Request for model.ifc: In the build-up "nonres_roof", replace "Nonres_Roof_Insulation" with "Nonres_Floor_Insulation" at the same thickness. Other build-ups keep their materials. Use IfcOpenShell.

First a look at what the model holds.

```python
import ifcopenshell
import ifcopenshell.util.element

model = ifcopenshell.open("model.ifc")
print(model.schema)
for layer_set in model.by_type("IfcMaterialLayerSet"):
    if layer_set.LayerSetName == "nonres_roof":
        for layer in layer_set.MaterialLayers:
            print(layer.id(), layer.Material and layer.Material.Name, layer.LayerThickness, sep=" | ")
        print(len(ifcopenshell.util.element.get_elements_by_material(model, layer_set)), "elements and types use it")
print(sorted(m.Name for m in model.by_type("IfcMaterial") if m.Name)[:60])
```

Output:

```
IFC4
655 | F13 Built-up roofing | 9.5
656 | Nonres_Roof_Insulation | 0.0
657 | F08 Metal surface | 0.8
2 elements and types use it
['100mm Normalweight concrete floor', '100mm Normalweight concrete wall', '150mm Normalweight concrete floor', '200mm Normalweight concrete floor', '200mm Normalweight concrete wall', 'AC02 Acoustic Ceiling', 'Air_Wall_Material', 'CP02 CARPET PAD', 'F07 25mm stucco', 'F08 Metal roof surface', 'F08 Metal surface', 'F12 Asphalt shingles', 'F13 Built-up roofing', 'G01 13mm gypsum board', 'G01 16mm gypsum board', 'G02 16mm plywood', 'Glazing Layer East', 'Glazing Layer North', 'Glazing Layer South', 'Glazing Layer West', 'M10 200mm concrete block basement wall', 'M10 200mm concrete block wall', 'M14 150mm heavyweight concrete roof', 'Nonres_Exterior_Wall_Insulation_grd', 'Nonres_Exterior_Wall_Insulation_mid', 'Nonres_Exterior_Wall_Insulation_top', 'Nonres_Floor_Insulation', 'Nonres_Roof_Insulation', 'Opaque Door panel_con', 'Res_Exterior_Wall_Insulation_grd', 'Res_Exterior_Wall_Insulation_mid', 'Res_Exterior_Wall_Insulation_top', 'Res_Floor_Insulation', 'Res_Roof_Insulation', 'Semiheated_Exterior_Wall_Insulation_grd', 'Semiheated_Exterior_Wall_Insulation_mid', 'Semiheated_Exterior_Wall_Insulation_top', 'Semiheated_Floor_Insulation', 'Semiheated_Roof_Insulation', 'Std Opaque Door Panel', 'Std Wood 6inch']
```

```python
import ifcopenshell
import ifcopenshell.api.material

model = ifcopenshell.open("model.ifc")

layer_set = next(s for s in model.by_type("IfcMaterialLayerSet") if s.LayerSetName == "nonres_roof")
layer = next(l for l in layer_set.MaterialLayers if l.Material and l.Material.Name == "Nonres_Roof_Insulation")
material = next(m for m in model.by_type("IfcMaterial") if m.Name == "Nonres_Floor_Insulation")

# Point this one layer at the other material; renaming the old one would change it everywhere.
ifcopenshell.api.material.edit_layer(model, layer=layer, attributes={}, material=material)

print([l.Material.Name if l.Material else None for l in layer_set.MaterialLayers])

model.write("model_updated.ifc")
```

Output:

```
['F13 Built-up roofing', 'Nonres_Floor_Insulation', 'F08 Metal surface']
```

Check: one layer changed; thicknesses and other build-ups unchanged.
